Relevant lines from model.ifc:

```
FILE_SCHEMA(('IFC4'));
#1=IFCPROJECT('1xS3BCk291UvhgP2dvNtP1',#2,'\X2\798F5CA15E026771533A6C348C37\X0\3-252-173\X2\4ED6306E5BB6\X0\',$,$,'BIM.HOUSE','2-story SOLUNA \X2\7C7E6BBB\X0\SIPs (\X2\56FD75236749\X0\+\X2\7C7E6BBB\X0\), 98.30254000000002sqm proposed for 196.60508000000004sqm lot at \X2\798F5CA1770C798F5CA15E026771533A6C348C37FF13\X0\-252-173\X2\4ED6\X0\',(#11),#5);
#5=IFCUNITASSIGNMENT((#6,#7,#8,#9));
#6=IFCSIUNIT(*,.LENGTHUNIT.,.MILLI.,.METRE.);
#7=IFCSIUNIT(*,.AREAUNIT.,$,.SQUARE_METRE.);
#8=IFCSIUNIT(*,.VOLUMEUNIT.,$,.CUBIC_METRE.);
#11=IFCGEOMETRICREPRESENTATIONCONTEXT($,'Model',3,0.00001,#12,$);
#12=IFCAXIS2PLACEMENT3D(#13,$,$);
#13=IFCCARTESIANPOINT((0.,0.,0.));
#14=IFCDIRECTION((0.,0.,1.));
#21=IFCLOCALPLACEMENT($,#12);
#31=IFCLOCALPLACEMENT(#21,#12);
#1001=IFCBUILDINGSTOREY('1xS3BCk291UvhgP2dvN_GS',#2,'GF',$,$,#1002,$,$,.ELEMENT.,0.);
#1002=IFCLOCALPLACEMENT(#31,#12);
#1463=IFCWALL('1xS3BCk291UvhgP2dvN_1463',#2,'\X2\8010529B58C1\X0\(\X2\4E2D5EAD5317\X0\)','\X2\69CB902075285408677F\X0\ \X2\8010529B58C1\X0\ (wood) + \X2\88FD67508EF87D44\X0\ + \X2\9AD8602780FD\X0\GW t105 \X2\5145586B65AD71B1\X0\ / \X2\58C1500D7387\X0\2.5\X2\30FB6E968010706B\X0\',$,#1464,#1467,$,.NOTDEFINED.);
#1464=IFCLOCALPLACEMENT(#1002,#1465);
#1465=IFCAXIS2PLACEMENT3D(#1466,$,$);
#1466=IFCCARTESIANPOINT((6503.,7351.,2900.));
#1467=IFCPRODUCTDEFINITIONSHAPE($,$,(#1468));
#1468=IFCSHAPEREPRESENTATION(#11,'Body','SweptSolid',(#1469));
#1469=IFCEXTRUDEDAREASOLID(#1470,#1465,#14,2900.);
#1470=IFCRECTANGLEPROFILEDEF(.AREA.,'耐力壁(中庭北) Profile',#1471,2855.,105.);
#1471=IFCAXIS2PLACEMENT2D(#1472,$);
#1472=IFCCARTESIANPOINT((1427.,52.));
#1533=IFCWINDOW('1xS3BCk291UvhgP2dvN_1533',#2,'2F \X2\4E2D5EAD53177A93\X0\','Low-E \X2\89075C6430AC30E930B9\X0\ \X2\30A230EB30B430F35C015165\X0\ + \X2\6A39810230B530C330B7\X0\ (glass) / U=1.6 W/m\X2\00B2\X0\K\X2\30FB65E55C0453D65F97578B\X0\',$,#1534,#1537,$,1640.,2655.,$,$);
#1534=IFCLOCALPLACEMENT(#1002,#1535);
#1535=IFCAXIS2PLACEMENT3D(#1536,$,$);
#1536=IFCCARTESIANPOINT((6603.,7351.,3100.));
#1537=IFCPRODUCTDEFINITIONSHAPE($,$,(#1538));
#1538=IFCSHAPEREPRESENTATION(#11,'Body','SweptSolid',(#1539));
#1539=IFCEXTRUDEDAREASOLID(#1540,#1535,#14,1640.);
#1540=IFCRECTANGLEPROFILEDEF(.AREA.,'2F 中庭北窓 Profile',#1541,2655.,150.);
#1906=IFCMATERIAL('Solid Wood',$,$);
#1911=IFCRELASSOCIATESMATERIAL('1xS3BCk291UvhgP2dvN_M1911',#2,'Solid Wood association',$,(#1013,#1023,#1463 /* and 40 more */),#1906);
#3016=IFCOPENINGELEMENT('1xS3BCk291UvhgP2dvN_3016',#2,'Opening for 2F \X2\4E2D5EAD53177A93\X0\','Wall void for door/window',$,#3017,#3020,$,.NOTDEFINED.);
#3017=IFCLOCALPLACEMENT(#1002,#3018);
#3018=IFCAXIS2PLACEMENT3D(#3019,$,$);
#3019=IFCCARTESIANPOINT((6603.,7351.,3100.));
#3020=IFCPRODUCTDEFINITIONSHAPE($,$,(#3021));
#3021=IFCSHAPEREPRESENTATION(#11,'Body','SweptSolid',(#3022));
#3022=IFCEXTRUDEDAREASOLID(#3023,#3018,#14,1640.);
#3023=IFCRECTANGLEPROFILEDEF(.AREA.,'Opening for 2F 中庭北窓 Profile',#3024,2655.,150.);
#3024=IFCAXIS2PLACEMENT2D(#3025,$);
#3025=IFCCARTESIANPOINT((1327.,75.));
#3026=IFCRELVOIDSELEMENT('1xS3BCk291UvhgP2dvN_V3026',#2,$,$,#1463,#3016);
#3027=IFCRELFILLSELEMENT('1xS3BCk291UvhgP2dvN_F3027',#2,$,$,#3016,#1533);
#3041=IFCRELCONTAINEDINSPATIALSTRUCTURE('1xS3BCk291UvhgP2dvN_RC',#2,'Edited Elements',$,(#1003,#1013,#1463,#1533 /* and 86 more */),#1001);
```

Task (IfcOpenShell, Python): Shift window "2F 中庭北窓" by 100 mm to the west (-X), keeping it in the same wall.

```python
import ifcopenshell
import ifcopenshell.api.geometry
import ifcopenshell.util.placement

model = ifcopenshell.open("model.ifc")

window = model.by_guid("1xS3BCk291UvhgP2dvN_1533")
opening = window.FillsVoids[0].RelatingOpeningElement
wall = opening.VoidsElements[0].RelatingBuildingElement

wall_matrix = ifcopenshell.util.placement.get_local_placement(wall.ObjectPlacement)
shift = wall_matrix[:3, 0] * -100.0
before = ifcopenshell.util.placement.get_local_placement(window.ObjectPlacement)[:3, 3].copy()

# The window is not placed relative to its opening, so move both.
for product in (opening, window):
    matrix = ifcopenshell.util.placement.get_local_placement(product.ObjectPlacement)
    matrix[:3, 3] += shift
    ifcopenshell.api.geometry.edit_object_placement(model, product=product, matrix=matrix, is_si=False)

after = ifcopenshell.util.placement.get_local_placement(window.ObjectPlacement)[:3, 3]
print("window moved by", (after - before).round(3) + 0.0)

model.write("model_rev.ifc")
```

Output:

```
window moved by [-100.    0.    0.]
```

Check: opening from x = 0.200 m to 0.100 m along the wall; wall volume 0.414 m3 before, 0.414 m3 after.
